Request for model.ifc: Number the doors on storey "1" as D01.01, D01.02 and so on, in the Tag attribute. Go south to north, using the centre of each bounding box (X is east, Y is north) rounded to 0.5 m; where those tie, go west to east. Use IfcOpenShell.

First a look at what the model holds.

```python
import ifcopenshell
import ifcopenshell.util.element
import ifcopenshell.util.placement

model = ifcopenshell.open("model.ifc")
print(model.schema)
storey = next(s for s in model.by_type("IfcBuildingStorey") if s.Name == "1")
doors = [e for e in ifcopenshell.util.element.get_decomposition(storey) if e.is_a("IfcDoor")]
for e in sorted(doors, key=lambda e: e.id()):
    origin = ifcopenshell.util.placement.get_local_placement(e.ObjectPlacement)[:3, 3]
    print(e.id(), e.Tag, e.Name, origin.round(2) + 0.0, sep=" | ")
```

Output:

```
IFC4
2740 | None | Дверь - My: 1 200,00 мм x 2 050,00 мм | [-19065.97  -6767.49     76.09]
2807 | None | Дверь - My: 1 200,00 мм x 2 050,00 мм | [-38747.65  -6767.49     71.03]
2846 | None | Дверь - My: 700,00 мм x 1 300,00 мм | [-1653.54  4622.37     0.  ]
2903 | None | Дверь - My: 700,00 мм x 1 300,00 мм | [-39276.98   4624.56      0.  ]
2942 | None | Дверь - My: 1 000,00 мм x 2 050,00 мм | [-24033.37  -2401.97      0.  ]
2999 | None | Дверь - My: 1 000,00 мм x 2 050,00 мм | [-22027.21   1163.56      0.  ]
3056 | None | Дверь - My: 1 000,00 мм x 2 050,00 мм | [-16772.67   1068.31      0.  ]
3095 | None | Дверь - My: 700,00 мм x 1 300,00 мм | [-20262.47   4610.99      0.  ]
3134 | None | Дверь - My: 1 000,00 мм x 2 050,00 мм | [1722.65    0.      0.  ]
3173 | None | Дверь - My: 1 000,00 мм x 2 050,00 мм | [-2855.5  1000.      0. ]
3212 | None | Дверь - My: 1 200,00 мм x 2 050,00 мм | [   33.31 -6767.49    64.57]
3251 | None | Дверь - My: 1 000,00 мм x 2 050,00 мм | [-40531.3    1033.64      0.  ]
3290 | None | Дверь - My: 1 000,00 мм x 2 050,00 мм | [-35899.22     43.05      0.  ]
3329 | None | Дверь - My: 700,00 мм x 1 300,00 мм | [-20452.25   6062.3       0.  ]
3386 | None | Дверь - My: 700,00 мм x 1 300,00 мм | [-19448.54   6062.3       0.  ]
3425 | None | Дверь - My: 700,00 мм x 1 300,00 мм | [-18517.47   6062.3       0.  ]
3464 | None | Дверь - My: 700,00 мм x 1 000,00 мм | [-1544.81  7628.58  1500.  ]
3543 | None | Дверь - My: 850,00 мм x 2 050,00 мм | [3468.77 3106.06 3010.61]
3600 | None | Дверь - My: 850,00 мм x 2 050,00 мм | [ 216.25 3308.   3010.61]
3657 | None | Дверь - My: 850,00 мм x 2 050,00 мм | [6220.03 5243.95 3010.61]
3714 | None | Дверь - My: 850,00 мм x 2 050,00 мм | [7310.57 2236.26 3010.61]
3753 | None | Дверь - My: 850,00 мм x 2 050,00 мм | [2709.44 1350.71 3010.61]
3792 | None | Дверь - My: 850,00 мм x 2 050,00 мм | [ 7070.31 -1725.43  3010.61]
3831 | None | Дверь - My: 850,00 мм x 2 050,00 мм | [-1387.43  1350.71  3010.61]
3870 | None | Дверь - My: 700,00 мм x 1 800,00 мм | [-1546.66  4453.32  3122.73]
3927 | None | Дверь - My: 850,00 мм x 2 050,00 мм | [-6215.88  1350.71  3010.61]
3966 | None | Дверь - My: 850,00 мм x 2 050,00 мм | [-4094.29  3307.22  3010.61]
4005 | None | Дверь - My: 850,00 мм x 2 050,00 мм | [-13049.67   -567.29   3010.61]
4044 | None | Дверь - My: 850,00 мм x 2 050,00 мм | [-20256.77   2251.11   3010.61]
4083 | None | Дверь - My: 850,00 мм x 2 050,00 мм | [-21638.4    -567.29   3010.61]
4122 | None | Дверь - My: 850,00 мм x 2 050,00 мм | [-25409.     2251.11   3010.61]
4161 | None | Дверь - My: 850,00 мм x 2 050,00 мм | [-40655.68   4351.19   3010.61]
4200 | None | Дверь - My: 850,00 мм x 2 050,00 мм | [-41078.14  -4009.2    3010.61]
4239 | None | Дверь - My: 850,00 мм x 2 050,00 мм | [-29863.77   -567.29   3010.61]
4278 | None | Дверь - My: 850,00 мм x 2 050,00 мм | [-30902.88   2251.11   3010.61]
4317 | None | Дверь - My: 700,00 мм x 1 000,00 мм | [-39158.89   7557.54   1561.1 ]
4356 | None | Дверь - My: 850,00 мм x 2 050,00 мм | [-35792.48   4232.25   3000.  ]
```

```python
import ifcopenshell
import ifcopenshell.geom
import ifcopenshell.util.element
import ifcopenshell.util.shape

model = ifcopenshell.open("model.ifc")
settings = ifcopenshell.geom.settings()
settings.set("use-world-coords", True)


def centre(element):
    shape = ifcopenshell.geom.create_shape(settings, element)
    return ifcopenshell.util.shape.get_bbox_centroid(shape.geometry)


storey = next(s for s in model.by_type("IfcBuildingStorey") if s.Name == "1")
doors = [e for e in ifcopenshell.util.element.get_decomposition(storey) if e.is_a("IfcDoor")]

# Insertion points can sit at a corner or the storey origin, so sort by the geometry (in metres).
centres = {e: centre(e) for e in doors}
doors.sort(key=lambda e: (round(centres[e][1] / 0.5), centres[e][0]))

for i, e in enumerate(doors, start=1):
    number = f"D01.{i:02d}"
    e.Tag = number
    print(e.id(), number)

model.write("model_edited.ifc")
```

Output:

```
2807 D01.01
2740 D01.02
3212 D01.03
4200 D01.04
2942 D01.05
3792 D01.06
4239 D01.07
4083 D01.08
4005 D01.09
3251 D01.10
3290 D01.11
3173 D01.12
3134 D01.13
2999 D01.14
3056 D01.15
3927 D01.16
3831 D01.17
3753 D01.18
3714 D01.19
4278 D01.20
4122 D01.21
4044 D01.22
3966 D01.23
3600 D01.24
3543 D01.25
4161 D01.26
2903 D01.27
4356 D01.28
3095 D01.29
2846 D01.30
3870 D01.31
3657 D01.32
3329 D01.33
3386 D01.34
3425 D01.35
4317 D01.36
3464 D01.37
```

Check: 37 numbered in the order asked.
